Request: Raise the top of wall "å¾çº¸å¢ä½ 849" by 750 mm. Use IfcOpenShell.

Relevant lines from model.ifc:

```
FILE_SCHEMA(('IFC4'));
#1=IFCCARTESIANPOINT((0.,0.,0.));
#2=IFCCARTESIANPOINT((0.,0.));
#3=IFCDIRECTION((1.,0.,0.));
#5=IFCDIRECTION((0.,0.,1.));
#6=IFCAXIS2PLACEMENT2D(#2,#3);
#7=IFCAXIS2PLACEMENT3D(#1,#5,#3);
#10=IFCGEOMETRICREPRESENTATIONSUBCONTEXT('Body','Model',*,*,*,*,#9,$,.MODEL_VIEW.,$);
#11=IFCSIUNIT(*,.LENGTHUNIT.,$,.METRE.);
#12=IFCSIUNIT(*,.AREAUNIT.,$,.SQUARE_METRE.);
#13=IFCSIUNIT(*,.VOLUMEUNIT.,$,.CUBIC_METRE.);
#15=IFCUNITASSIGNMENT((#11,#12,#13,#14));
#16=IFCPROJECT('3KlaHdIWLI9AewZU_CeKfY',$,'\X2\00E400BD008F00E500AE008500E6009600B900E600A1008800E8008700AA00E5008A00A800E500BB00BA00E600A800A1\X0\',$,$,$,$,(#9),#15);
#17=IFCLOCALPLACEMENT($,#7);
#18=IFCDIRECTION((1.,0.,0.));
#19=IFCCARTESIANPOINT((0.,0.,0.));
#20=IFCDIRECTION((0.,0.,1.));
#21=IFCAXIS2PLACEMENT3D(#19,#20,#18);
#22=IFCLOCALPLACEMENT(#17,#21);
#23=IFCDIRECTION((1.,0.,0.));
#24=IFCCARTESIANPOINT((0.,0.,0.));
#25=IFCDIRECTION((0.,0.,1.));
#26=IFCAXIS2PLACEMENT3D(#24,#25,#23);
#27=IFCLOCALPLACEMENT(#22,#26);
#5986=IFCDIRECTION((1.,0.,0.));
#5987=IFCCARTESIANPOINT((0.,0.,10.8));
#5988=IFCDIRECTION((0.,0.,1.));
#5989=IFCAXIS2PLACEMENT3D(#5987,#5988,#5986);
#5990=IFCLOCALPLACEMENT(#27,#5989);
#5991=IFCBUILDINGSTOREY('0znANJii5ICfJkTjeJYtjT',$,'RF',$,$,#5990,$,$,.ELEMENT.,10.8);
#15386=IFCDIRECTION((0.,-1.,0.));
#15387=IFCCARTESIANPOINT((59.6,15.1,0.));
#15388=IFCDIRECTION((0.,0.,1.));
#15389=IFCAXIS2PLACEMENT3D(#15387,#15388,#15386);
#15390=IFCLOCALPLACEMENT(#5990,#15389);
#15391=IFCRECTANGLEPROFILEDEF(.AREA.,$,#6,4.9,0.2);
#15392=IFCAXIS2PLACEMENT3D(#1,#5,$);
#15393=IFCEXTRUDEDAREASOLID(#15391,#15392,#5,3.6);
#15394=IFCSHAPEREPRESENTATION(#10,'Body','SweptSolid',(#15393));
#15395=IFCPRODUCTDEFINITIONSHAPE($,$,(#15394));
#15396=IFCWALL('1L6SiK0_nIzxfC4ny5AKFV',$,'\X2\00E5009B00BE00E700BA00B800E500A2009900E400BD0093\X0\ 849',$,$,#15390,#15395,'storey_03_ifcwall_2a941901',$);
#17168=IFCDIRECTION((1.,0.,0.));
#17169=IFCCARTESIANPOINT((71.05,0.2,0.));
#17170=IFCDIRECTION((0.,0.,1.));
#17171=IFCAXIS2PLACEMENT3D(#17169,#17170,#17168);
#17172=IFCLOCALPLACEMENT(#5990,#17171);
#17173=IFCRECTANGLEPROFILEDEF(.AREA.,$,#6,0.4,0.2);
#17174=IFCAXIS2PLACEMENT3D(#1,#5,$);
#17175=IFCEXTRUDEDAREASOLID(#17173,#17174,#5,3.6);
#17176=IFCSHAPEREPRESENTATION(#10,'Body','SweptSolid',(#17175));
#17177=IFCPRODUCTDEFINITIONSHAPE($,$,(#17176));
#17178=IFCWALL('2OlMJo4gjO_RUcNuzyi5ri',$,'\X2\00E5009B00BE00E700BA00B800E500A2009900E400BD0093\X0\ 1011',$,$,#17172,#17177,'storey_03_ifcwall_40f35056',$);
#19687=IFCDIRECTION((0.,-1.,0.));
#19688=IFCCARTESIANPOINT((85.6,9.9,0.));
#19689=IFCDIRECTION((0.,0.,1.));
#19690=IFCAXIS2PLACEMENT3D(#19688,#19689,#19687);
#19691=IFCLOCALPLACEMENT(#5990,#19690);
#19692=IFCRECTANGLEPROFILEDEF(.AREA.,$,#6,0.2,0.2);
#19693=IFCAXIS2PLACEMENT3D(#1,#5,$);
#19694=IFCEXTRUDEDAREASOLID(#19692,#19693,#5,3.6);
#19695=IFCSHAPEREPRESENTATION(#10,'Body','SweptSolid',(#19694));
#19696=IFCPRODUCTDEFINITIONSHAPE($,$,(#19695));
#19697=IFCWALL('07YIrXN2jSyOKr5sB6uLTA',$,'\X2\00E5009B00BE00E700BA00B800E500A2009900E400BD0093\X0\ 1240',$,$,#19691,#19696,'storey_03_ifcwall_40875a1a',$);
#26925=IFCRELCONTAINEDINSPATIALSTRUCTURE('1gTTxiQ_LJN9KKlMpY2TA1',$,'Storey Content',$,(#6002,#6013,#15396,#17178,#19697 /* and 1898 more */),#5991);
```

```python
import ifcopenshell
import ifcopenshell.geom
import ifcopenshell.util.representation
import ifcopenshell.util.shape
import ifcopenshell.util.unit

model = ifcopenshell.open("model.ifc")
unit_scale = ifcopenshell.util.unit.calculate_unit_scale(model)
settings = ifcopenshell.geom.settings()


def volume(element):
    """Net volume in cubic metres, openings subtracted."""
    shape = ifcopenshell.geom.create_shape(settings, element)
    return ifcopenshell.util.shape.get_volume(shape.geometry)


wall = model.by_guid("1L6SiK0_nIzxfC4ny5AKFV")
before = volume(wall)

body = ifcopenshell.util.representation.get_representation(wall, "Model", "Body")
solid = body.Items[0]
old_height = solid.Depth
solid.Depth += 0.75 / unit_scale
after = volume(wall)

print(f"height {old_height:g} -> {solid.Depth:g}, volume {before:.3f} -> {after:.3f} m3")

model.write("model_updated.ifc")
```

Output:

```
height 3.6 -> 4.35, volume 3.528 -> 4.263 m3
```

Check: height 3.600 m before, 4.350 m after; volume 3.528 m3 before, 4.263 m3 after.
